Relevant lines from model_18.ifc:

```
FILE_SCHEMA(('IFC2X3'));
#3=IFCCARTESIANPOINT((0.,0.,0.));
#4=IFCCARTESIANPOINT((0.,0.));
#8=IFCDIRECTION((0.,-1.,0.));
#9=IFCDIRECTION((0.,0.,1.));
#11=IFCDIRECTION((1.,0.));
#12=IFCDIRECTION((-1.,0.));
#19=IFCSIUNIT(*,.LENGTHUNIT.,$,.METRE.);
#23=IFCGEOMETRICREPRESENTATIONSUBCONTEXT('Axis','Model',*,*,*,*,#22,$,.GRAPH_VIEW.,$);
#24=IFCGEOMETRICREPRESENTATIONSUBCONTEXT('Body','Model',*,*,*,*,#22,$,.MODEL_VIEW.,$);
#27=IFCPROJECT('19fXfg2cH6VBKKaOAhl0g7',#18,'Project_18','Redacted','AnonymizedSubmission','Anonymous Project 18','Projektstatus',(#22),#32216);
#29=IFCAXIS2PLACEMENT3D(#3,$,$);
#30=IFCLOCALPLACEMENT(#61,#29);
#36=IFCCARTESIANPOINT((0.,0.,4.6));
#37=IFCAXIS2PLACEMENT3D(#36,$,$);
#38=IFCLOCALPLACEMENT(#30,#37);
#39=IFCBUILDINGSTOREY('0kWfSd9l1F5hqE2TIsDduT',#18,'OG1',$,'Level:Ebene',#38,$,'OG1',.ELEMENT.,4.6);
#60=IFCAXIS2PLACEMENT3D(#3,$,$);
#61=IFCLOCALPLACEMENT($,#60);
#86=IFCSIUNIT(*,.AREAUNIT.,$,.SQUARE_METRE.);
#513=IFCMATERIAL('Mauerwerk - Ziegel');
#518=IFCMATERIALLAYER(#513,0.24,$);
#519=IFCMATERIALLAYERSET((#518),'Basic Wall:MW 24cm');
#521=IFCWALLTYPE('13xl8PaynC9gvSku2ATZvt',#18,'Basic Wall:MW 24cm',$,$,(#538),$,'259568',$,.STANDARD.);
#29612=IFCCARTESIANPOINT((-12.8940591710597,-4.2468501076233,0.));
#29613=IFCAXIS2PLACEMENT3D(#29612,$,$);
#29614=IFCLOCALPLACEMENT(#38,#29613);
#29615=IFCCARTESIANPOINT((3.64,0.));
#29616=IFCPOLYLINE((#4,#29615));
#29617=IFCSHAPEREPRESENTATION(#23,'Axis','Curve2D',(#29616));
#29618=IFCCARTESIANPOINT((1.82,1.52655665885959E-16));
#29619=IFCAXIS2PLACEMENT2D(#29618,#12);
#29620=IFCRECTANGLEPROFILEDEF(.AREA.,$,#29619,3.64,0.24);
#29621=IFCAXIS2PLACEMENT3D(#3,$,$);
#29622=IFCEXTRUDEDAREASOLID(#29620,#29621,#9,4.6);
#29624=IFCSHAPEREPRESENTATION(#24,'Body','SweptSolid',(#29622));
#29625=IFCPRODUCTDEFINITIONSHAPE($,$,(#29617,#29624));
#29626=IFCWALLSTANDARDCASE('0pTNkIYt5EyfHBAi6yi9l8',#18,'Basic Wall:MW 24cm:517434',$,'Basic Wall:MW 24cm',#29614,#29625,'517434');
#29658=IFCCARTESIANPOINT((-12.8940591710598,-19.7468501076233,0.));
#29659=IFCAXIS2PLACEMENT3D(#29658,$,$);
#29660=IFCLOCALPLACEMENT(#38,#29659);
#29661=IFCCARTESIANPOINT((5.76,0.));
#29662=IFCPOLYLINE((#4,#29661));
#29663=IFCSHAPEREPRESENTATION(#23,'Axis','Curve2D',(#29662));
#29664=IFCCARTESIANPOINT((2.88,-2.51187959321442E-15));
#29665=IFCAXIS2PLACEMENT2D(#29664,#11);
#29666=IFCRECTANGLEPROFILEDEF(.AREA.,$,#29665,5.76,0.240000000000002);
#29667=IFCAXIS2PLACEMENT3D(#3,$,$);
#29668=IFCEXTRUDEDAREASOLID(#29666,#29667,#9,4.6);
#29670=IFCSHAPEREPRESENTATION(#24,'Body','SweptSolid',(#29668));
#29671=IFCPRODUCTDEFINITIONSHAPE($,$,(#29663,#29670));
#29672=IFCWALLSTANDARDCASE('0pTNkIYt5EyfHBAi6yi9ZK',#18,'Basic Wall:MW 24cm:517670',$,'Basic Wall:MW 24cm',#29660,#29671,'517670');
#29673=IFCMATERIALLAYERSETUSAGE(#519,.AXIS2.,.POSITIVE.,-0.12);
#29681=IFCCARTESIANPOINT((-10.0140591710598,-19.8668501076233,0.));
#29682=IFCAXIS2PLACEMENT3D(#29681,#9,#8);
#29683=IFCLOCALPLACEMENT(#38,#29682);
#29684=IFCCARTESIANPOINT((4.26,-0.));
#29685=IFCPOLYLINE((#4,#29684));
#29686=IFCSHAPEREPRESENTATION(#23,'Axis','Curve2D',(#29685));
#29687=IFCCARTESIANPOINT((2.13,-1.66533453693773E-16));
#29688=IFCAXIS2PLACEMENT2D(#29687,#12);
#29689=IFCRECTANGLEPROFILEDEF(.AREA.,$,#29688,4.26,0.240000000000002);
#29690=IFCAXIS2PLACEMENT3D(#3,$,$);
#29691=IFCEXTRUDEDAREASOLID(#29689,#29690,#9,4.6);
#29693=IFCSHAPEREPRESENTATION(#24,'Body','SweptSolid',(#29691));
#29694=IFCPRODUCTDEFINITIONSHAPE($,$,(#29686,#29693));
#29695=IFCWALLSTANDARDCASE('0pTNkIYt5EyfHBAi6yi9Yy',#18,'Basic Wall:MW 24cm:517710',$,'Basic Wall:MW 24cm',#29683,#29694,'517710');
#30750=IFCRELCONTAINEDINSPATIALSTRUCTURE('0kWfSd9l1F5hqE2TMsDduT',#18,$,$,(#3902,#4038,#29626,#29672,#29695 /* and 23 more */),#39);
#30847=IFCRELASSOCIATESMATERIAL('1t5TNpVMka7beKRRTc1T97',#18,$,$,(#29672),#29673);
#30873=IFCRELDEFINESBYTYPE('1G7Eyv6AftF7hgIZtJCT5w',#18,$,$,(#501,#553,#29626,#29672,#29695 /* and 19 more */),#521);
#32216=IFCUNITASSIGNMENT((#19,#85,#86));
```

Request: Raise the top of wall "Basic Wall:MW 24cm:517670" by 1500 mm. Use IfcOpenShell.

```python
import ifcopenshell
import ifcopenshell.geom
import ifcopenshell.util.representation
import ifcopenshell.util.shape
import ifcopenshell.util.unit

model = ifcopenshell.open("model_18.ifc")
unit_scale = ifcopenshell.util.unit.calculate_unit_scale(model)
settings = ifcopenshell.geom.settings()


def volume(element):
    """Net volume in cubic metres, openings subtracted."""
    shape = ifcopenshell.geom.create_shape(settings, element)
    return ifcopenshell.util.shape.get_volume(shape.geometry)


wall = model.by_id(29672)
before = volume(wall)

body = ifcopenshell.util.representation.get_representation(wall, "Model", "Body")
solid = body.Items[0]
old_height = solid.Depth
solid.Depth += 1.5 / unit_scale
after = volume(wall)

print(f"height {old_height:g} -> {solid.Depth:g}, volume {before:.3f} -> {after:.3f} m3")

model.write("model_18_rev.ifc")
```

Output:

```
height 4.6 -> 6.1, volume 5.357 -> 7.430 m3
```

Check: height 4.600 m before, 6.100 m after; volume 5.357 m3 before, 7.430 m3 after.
